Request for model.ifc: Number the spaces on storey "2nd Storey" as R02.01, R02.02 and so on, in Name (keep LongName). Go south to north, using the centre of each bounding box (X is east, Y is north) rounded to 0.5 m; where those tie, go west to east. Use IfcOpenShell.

First a look at what the model holds.

```python
import ifcopenshell
import ifcopenshell.util.element
import ifcopenshell.util.placement

model = ifcopenshell.open("model.ifc")
print(model.schema)
storey = next(s for s in model.by_type("IfcBuildingStorey") if s.Name == "2nd Storey")
spaces = [e for e in ifcopenshell.util.element.get_decomposition(storey) if e.is_a("IfcSpace")]
for e in sorted(spaces, key=lambda e: e.id()):
    origin = ifcopenshell.util.placement.get_local_placement(e.ObjectPlacement)[:3, 3]
    print(e.id(), e.Name, e.LongName, origin.round(2) + 0.0, sep=" | ")
```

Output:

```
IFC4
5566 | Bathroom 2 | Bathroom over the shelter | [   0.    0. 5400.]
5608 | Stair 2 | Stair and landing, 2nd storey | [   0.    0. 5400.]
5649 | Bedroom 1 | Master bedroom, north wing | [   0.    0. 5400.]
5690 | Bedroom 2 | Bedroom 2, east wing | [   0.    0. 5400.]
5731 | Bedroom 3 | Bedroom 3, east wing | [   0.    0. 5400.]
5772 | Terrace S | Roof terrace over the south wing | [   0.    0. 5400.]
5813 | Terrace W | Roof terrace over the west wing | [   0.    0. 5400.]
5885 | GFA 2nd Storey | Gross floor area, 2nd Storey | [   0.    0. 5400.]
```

```python
import ifcopenshell
import ifcopenshell.geom
import ifcopenshell.util.element
import ifcopenshell.util.shape

model = ifcopenshell.open("model.ifc")
settings = ifcopenshell.geom.settings()
settings.set("use-world-coords", True)


def centre(element):
    shape = ifcopenshell.geom.create_shape(settings, element)
    return ifcopenshell.util.shape.get_bbox_centroid(shape.geometry)


storey = next(s for s in model.by_type("IfcBuildingStorey") if s.Name == "2nd Storey")
spaces = [e for e in ifcopenshell.util.element.get_decomposition(storey) if e.is_a("IfcSpace")]

# Insertion points can sit at a corner or the storey origin, so sort by the geometry (in metres).
centres = {e: centre(e) for e in spaces}
spaces.sort(key=lambda e: (round(centres[e][1] / 0.5), centres[e][0]))

for i, e in enumerate(spaces, start=1):
    number = f"R02.{i:02d}"
    e.Name = number
    print(e.id(), number)

model.write("model-out.ifc")
```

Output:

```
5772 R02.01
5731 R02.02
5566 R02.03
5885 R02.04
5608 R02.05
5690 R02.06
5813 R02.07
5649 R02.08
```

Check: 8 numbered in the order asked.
